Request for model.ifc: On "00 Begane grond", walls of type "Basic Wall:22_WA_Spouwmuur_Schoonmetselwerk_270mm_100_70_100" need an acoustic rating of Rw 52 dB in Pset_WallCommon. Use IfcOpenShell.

First a look at what the model holds.

```python
import ifcopenshell
import ifcopenshell.util.element

model = ifcopenshell.open("model.ifc")
print(model.schema)
storey = next(s for s in model.by_type("IfcBuildingStorey") if s.Name == "00 Begane grond")
walls = [e for e in ifcopenshell.util.element.get_decomposition(storey) if e.is_a("IfcWall")]
seen = {}
for e in walls:
    element_type = ifcopenshell.util.element.get_type(e)
    key = (element_type.Name if element_type != e and element_type else None, ifcopenshell.util.element.get_pset(e, "Pset_WallCommon", "AcousticRating"))
    seen[key] = seen.get(key, 0) + 1
for (name, value), count in sorted(seen.items(), key=str):
    print(count, "x", name, "|", value)
```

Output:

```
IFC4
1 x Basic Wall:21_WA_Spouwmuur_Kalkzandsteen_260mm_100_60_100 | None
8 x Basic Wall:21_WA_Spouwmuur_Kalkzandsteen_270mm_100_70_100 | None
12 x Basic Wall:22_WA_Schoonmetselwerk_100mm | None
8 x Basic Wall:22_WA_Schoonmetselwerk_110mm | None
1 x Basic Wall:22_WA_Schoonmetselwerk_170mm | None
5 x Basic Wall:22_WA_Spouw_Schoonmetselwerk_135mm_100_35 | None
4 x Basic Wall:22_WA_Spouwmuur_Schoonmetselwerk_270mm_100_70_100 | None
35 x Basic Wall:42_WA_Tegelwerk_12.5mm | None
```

```python
import ifcopenshell
import ifcopenshell.api.pset
import ifcopenshell.util.element

model = ifcopenshell.open("model.ifc")

storey = next(s for s in model.by_type("IfcBuildingStorey") if s.Name == "00 Begane grond")
walls = [e for e in ifcopenshell.util.element.get_decomposition(storey) if e.is_a("IfcWall")]

count = 0
for e in walls:
    element_type = ifcopenshell.util.element.get_type(e)
    if element_type in (None, e) or element_type.Name != "Basic Wall:22_WA_Spouwmuur_Schoonmetselwerk_270mm_100_70_100":
        continue
    # add_pset returns the element's existing set when there is one.
    pset = ifcopenshell.api.pset.add_pset(model, product=e, name="Pset_WallCommon")
    ifcopenshell.api.pset.edit_pset(model, pset=pset, properties={"AcousticRating": "Rw 52 dB"})
    count += 1

print(count, "walls updated")

model.write("model_v2.ifc")
```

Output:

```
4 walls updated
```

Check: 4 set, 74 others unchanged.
